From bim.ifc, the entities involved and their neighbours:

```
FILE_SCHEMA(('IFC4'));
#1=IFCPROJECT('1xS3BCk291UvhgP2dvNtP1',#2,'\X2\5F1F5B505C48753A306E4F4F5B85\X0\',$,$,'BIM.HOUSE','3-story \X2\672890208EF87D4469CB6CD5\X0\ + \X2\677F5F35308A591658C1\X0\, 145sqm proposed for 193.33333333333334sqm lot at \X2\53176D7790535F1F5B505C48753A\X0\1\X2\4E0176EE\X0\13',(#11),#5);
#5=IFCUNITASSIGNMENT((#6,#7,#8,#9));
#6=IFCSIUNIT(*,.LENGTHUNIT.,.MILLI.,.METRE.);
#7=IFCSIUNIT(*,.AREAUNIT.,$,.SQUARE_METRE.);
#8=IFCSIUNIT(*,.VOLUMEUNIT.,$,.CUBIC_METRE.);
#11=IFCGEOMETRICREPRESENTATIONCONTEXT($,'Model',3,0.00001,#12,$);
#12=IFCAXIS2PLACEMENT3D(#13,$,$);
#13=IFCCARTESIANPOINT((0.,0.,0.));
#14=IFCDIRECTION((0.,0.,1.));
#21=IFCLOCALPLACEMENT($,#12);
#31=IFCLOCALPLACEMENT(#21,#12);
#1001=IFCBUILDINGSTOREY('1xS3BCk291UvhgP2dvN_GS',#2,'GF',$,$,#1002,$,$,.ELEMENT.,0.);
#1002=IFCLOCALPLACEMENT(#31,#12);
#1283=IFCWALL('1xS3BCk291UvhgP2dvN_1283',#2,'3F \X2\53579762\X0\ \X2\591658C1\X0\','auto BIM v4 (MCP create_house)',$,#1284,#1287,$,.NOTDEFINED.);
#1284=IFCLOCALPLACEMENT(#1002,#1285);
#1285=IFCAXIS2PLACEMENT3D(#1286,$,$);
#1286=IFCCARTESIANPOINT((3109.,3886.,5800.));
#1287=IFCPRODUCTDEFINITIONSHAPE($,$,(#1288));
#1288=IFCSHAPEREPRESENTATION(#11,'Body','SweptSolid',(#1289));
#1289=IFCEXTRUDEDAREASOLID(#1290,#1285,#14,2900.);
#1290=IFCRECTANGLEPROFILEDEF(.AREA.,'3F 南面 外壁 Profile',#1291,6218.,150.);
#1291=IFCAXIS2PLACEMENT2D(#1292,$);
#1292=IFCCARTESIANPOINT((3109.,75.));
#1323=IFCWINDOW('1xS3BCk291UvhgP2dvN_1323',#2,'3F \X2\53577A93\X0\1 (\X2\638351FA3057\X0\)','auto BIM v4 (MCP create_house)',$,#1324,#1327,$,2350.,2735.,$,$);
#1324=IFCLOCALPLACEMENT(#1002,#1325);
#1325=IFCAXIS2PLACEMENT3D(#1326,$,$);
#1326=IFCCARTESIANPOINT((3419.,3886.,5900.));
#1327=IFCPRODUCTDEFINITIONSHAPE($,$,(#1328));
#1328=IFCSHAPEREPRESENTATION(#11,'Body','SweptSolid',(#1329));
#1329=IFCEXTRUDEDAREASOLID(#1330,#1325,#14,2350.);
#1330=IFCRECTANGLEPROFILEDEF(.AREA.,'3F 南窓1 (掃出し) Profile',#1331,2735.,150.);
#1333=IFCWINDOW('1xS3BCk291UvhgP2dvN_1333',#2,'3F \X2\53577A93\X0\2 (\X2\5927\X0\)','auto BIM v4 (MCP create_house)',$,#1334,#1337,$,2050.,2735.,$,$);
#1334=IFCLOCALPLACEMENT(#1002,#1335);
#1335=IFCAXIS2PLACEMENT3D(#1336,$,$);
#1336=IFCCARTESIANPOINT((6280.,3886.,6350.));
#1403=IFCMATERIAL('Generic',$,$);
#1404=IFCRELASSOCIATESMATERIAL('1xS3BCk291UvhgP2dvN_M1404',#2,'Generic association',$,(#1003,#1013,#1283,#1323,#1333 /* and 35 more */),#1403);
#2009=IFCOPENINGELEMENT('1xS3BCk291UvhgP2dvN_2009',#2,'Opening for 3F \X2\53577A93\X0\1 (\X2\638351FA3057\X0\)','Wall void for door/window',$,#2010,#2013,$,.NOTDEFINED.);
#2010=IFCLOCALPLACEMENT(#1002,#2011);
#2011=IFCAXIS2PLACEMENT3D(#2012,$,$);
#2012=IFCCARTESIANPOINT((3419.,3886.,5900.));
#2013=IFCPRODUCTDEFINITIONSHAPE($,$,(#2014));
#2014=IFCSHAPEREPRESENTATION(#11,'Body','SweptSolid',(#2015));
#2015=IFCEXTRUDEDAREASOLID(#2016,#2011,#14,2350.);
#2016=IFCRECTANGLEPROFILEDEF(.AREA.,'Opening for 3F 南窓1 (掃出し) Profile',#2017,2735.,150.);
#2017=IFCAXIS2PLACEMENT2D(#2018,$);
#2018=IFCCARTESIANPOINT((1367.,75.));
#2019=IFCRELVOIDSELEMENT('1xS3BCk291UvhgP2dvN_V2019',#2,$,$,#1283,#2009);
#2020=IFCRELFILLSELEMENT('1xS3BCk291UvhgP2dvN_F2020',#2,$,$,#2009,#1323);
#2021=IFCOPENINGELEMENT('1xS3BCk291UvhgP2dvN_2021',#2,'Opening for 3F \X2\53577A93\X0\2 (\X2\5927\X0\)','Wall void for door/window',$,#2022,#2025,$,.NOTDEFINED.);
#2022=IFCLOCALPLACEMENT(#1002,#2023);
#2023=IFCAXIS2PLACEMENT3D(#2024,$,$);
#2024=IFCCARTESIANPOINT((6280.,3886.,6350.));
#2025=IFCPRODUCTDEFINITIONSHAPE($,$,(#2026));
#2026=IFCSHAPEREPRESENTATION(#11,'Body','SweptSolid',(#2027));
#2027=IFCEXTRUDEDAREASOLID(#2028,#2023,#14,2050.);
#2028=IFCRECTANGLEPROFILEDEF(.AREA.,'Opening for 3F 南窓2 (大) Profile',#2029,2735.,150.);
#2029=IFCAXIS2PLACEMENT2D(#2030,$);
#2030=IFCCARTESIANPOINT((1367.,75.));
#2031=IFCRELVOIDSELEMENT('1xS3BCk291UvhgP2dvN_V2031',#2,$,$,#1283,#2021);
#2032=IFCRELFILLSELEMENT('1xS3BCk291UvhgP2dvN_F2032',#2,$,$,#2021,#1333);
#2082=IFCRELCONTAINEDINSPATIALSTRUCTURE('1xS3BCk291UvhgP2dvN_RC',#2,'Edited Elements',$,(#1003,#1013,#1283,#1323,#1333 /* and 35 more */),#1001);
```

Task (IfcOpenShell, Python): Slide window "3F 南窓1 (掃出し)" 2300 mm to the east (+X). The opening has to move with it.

```python
import ifcopenshell
import ifcopenshell.api.geometry
import ifcopenshell.util.placement
import ifcopenshell.util.unit

model = ifcopenshell.open("bim.ifc")
unit_scale = ifcopenshell.util.unit.calculate_unit_scale(model)

window = model.by_guid("1xS3BCk291UvhgP2dvN_1323")
opening = window.FillsVoids[0].RelatingOpeningElement
wall = opening.VoidsElements[0].RelatingBuildingElement

wall_matrix = ifcopenshell.util.placement.get_local_placement(wall.ObjectPlacement)
shift = wall_matrix[:3, 0] * 2.3 / unit_scale
before = ifcopenshell.util.placement.get_local_placement(window.ObjectPlacement)[:3, 3].copy()

# The window is not placed relative to its opening, so move both.
for product in (opening, window):
    matrix = ifcopenshell.util.placement.get_local_placement(product.ObjectPlacement)
    matrix[:3, 3] += shift
    ifcopenshell.api.geometry.edit_object_placement(model, product=product, matrix=matrix, is_si=False)

after = ifcopenshell.util.placement.get_local_placement(window.ObjectPlacement)[:3, 3]
print("window moved by", (after - before).round(3) + 0.0)

model.write("bim_updated.ifc")
```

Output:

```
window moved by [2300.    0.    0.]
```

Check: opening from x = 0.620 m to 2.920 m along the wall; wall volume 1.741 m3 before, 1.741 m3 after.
